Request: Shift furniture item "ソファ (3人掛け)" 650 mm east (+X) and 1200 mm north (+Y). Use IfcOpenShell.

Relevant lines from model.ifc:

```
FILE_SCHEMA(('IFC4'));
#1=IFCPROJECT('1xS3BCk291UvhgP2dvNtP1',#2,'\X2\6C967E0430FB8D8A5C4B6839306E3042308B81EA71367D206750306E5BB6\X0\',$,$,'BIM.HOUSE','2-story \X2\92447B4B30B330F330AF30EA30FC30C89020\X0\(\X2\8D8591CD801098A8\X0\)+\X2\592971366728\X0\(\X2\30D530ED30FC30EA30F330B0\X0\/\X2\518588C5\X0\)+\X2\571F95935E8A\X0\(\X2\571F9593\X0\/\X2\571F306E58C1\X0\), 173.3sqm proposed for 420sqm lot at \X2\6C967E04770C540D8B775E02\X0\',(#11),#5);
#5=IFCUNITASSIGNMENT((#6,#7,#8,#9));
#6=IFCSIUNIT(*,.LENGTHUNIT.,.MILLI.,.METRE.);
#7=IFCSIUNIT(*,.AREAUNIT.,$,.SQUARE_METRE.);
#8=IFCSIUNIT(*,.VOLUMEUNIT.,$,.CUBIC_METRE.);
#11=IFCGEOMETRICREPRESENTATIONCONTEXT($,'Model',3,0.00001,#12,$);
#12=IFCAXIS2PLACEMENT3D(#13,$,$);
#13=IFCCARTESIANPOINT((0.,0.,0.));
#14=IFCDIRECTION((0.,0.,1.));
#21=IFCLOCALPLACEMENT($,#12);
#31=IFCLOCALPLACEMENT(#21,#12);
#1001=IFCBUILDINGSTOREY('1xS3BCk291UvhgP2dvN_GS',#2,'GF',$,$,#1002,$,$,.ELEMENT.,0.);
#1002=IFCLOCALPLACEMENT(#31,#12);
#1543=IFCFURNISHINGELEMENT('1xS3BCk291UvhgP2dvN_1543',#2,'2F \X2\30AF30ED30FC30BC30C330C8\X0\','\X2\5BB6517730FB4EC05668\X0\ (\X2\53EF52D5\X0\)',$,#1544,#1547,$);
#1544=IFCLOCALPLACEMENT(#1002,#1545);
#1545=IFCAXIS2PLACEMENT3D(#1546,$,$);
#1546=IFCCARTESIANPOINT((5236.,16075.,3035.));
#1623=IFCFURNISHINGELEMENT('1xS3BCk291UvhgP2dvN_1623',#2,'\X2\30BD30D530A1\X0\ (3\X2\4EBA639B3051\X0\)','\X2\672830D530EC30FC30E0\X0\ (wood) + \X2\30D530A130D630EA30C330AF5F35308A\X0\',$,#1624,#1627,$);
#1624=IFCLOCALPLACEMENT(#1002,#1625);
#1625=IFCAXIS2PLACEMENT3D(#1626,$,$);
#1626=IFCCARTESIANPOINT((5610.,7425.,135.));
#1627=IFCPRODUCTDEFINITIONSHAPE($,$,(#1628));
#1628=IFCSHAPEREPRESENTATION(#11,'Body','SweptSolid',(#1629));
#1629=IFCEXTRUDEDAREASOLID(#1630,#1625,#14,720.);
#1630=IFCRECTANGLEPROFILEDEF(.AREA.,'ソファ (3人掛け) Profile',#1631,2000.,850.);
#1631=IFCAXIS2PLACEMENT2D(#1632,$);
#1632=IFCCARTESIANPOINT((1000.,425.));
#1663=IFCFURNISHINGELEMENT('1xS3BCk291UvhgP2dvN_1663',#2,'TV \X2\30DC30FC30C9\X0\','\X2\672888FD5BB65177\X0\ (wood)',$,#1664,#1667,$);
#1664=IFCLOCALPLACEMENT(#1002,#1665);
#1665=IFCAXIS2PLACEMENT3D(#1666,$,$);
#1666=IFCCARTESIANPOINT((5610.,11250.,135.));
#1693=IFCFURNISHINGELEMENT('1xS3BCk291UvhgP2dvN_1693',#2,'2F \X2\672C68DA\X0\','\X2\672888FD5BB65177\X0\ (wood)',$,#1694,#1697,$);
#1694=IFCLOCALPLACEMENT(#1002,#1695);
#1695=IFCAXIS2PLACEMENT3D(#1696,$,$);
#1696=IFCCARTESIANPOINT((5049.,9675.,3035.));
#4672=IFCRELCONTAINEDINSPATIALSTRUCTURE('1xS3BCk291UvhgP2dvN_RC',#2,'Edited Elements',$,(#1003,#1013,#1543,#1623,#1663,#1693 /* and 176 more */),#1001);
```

```python
import ifcopenshell
import ifcopenshell.api.geometry
import ifcopenshell.util.placement

model = ifcopenshell.open("model.ifc")

item = model.by_guid("1xS3BCk291UvhgP2dvN_1623")
matrix = ifcopenshell.util.placement.get_local_placement(item.ObjectPlacement)
matrix[0, 3] += 650.0
matrix[1, 3] += 1200.0
ifcopenshell.api.geometry.edit_object_placement(model, product=item, matrix=matrix, is_si=False)

print(ifcopenshell.util.placement.get_local_placement(item.ObjectPlacement).round(3) + 0.0)

model.write("model_edited.ifc")
```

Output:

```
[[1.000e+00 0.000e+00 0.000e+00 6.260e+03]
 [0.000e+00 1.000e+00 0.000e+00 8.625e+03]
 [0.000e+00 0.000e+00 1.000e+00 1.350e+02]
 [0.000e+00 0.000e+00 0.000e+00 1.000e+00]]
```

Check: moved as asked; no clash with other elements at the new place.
